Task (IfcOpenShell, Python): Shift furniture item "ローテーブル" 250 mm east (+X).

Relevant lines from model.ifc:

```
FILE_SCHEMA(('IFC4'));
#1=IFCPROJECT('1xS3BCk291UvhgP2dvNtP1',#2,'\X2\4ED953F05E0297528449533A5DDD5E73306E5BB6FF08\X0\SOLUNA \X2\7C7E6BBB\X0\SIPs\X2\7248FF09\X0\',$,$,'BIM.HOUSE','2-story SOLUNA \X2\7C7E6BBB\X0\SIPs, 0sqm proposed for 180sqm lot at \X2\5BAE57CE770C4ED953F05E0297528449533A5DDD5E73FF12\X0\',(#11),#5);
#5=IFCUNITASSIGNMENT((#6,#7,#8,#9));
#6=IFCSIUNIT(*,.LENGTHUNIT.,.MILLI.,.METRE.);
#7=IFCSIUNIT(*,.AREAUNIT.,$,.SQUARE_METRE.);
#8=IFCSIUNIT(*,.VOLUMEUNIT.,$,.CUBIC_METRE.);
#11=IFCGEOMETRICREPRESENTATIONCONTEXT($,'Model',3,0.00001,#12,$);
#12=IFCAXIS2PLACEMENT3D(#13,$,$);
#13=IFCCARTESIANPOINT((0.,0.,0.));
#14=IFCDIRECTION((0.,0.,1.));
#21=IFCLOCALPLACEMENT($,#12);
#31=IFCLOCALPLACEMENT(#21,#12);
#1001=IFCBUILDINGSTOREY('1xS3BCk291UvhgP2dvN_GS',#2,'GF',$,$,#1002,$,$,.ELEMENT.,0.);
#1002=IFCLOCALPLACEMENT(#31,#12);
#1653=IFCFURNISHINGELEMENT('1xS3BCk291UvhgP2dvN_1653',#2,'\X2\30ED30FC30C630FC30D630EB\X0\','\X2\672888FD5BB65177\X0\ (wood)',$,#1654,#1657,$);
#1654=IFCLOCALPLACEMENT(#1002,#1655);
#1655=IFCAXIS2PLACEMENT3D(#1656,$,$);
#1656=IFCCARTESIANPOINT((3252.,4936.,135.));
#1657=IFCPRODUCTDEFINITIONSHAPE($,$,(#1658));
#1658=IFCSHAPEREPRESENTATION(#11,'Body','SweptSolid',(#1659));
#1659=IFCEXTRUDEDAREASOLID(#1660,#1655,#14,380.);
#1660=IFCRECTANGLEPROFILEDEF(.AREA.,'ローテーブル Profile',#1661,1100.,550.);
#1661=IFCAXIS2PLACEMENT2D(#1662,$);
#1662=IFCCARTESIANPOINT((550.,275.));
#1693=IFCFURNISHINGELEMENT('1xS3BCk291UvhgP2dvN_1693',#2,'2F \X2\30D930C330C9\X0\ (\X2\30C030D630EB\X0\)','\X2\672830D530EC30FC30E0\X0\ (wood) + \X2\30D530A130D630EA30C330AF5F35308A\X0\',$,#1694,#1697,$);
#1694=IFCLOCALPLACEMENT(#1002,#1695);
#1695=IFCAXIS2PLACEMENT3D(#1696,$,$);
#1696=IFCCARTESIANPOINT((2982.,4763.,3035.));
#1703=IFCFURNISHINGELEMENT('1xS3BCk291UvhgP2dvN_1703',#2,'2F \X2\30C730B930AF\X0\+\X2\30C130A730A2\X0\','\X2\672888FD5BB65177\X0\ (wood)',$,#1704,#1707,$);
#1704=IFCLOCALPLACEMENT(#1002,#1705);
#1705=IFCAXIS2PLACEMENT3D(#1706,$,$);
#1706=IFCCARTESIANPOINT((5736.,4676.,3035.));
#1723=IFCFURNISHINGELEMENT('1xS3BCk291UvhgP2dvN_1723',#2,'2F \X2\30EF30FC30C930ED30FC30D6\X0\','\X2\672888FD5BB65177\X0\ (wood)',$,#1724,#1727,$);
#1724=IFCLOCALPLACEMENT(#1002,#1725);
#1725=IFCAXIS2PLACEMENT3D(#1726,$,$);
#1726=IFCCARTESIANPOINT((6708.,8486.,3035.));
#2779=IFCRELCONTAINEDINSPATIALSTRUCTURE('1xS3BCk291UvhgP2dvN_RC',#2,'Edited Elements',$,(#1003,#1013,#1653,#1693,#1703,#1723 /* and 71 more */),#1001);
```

```python
import ifcopenshell
import ifcopenshell.api.geometry
import ifcopenshell.util.placement
import ifcopenshell.util.unit

model = ifcopenshell.open("model.ifc")
unit_scale = ifcopenshell.util.unit.calculate_unit_scale(model)

item = model.by_guid("1xS3BCk291UvhgP2dvN_1653")
matrix = ifcopenshell.util.placement.get_local_placement(item.ObjectPlacement)
matrix[0, 3] += 0.25 / unit_scale
ifcopenshell.api.geometry.edit_object_placement(model, product=item, matrix=matrix, is_si=False)

print(ifcopenshell.util.placement.get_local_placement(item.ObjectPlacement).round(3) + 0.0)

model.write("model_rev.ifc")
```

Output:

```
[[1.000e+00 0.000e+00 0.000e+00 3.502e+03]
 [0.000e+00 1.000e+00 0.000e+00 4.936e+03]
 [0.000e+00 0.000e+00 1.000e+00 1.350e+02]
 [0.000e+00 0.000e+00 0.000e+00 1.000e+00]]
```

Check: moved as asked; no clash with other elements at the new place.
